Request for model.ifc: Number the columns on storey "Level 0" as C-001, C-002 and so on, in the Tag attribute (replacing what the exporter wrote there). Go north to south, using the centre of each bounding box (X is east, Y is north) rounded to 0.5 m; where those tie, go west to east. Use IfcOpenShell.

First a look at what the model holds.

```python
import ifcopenshell
import ifcopenshell.util.element
import ifcopenshell.util.placement

model = ifcopenshell.open("model.ifc")
print(model.schema)
storey = next(s for s in model.by_type("IfcBuildingStorey") if s.Name == "Level 0")
columns = [e for e in ifcopenshell.util.element.get_decomposition(storey) if e.is_a("IfcColumn")]
for e in sorted(columns, key=lambda e: e.id()):
    origin = ifcopenshell.util.placement.get_local_placement(e.ObjectPlacement)[:3, 3]
    print(e.id(), e.Tag, e.Name, origin.round(2) + 0.0, sep=" | ")
```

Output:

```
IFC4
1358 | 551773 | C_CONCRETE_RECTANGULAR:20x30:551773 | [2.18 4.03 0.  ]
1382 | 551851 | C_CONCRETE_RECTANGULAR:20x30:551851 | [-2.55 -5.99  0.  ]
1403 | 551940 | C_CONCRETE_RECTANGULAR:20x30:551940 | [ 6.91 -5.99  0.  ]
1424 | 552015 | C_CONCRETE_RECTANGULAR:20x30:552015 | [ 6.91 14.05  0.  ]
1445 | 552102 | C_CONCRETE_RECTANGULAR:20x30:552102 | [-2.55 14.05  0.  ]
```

```python
import ifcopenshell
import ifcopenshell.geom
import ifcopenshell.util.element
import ifcopenshell.util.shape

model = ifcopenshell.open("model.ifc")
settings = ifcopenshell.geom.settings()
settings.set("use-world-coords", True)


def centre(element):
    shape = ifcopenshell.geom.create_shape(settings, element)
    return ifcopenshell.util.shape.get_bbox_centroid(shape.geometry)


storey = next(s for s in model.by_type("IfcBuildingStorey") if s.Name == "Level 0")
columns = [e for e in ifcopenshell.util.element.get_decomposition(storey) if e.is_a("IfcColumn")]

# Insertion points can sit at a corner or the storey origin, so sort by the geometry (in metres).
centres = {e: centre(e) for e in columns}
columns.sort(key=lambda e: (-round(centres[e][1] / 0.5), centres[e][0]))

for i, e in enumerate(columns, start=1):
    number = f"C-0{i:02d}"
    e.Tag = number
    print(e.id(), number)

model.write("model-out.ifc")
```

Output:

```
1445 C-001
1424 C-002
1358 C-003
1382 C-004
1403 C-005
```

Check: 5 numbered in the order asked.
